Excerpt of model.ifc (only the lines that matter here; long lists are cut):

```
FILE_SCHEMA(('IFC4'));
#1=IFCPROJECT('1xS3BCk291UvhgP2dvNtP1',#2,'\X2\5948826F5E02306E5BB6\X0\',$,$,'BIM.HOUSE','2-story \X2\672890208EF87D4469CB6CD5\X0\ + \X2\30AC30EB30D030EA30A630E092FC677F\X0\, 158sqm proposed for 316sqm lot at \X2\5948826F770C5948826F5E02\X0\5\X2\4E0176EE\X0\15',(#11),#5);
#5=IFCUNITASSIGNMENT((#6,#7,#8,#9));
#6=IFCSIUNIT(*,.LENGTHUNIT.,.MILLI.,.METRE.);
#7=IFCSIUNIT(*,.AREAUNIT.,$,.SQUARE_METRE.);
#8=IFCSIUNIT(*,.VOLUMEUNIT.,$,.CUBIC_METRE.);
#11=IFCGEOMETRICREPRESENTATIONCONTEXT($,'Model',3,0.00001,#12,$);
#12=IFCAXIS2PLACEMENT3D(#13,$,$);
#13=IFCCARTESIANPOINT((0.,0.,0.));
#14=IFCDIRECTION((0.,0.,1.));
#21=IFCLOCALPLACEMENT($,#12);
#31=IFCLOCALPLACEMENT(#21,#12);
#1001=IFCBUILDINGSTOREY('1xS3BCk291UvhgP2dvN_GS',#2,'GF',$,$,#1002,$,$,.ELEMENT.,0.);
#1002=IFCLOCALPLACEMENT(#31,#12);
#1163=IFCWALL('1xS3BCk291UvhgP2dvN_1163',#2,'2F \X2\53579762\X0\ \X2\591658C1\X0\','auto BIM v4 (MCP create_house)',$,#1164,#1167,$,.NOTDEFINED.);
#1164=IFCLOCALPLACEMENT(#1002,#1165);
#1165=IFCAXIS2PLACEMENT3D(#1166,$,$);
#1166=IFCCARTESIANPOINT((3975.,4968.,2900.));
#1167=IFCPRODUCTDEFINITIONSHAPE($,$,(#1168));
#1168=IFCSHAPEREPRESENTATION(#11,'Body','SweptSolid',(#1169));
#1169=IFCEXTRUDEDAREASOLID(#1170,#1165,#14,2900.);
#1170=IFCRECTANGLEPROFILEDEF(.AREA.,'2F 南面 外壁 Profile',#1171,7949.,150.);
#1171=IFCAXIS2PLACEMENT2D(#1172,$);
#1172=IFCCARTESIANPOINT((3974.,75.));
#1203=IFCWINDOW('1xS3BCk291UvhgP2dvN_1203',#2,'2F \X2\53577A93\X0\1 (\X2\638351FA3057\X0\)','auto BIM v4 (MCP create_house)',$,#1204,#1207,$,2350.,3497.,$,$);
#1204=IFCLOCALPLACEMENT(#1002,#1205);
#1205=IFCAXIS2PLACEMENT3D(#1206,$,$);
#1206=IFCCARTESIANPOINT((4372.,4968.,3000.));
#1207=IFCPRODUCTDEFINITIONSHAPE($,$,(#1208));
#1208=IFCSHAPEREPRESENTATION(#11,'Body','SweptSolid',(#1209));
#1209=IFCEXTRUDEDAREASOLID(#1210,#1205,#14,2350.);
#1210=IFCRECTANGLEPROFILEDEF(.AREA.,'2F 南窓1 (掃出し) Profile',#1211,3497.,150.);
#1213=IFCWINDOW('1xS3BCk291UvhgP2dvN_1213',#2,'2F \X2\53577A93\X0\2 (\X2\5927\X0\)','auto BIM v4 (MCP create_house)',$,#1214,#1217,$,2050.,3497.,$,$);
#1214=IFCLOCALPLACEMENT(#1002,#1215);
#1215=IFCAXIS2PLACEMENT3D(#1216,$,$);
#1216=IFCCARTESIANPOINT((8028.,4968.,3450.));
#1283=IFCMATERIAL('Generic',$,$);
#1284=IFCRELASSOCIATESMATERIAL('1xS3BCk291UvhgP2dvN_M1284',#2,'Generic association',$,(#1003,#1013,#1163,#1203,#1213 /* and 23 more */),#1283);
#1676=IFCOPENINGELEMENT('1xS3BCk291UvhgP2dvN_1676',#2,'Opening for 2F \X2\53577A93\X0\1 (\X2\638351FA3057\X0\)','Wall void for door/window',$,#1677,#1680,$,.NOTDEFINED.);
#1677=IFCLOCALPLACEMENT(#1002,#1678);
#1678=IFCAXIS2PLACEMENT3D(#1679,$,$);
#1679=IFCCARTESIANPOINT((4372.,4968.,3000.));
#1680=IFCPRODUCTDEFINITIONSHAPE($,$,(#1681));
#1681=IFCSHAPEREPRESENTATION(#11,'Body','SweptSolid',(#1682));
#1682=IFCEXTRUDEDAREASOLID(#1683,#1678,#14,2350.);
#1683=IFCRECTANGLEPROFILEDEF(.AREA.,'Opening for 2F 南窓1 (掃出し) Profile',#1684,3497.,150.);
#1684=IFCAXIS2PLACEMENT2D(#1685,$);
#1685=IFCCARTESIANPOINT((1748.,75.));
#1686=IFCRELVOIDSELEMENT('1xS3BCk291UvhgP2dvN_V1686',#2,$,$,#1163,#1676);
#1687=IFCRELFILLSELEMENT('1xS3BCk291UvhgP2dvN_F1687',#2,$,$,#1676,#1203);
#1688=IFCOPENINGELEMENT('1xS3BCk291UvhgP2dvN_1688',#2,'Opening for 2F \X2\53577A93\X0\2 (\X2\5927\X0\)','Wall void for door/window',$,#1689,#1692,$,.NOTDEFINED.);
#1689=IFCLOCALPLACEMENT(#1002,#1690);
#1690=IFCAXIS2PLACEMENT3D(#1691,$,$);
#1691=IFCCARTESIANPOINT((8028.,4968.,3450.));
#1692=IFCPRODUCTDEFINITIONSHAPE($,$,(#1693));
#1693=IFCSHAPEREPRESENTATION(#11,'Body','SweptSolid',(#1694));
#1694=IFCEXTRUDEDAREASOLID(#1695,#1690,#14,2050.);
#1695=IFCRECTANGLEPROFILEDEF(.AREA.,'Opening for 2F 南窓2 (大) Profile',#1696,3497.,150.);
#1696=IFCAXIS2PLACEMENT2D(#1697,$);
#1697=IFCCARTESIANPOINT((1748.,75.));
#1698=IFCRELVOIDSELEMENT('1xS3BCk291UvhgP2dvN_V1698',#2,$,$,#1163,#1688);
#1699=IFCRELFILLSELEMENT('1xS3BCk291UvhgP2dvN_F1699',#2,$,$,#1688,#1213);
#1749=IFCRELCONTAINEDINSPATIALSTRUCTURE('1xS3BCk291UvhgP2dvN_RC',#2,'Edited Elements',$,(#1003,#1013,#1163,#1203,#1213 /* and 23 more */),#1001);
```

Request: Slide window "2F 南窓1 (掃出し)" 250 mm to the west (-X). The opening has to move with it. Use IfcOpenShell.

```python
import ifcopenshell
import ifcopenshell.api.geometry
import ifcopenshell.util.placement

model = ifcopenshell.open("model.ifc")

window = model.by_id(1203)
opening = window.FillsVoids[0].RelatingOpeningElement
wall = opening.VoidsElements[0].RelatingBuildingElement

wall_matrix = ifcopenshell.util.placement.get_local_placement(wall.ObjectPlacement)
shift = wall_matrix[:3, 0] * -250.0
before = ifcopenshell.util.placement.get_local_placement(window.ObjectPlacement)[:3, 3].copy()

# The window is not placed relative to its opening, so move both.
for product in (opening, window):
    matrix = ifcopenshell.util.placement.get_local_placement(product.ObjectPlacement)
    matrix[:3, 3] += shift
    ifcopenshell.api.geometry.edit_object_placement(model, product=product, matrix=matrix, is_si=False)

after = ifcopenshell.util.placement.get_local_placement(window.ObjectPlacement)[:3, 3]
print("window moved by", (after - before).round(3) + 0.0)

model.write("model-out.ifc")
```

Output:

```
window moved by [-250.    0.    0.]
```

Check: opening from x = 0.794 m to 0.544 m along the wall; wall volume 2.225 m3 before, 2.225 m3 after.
